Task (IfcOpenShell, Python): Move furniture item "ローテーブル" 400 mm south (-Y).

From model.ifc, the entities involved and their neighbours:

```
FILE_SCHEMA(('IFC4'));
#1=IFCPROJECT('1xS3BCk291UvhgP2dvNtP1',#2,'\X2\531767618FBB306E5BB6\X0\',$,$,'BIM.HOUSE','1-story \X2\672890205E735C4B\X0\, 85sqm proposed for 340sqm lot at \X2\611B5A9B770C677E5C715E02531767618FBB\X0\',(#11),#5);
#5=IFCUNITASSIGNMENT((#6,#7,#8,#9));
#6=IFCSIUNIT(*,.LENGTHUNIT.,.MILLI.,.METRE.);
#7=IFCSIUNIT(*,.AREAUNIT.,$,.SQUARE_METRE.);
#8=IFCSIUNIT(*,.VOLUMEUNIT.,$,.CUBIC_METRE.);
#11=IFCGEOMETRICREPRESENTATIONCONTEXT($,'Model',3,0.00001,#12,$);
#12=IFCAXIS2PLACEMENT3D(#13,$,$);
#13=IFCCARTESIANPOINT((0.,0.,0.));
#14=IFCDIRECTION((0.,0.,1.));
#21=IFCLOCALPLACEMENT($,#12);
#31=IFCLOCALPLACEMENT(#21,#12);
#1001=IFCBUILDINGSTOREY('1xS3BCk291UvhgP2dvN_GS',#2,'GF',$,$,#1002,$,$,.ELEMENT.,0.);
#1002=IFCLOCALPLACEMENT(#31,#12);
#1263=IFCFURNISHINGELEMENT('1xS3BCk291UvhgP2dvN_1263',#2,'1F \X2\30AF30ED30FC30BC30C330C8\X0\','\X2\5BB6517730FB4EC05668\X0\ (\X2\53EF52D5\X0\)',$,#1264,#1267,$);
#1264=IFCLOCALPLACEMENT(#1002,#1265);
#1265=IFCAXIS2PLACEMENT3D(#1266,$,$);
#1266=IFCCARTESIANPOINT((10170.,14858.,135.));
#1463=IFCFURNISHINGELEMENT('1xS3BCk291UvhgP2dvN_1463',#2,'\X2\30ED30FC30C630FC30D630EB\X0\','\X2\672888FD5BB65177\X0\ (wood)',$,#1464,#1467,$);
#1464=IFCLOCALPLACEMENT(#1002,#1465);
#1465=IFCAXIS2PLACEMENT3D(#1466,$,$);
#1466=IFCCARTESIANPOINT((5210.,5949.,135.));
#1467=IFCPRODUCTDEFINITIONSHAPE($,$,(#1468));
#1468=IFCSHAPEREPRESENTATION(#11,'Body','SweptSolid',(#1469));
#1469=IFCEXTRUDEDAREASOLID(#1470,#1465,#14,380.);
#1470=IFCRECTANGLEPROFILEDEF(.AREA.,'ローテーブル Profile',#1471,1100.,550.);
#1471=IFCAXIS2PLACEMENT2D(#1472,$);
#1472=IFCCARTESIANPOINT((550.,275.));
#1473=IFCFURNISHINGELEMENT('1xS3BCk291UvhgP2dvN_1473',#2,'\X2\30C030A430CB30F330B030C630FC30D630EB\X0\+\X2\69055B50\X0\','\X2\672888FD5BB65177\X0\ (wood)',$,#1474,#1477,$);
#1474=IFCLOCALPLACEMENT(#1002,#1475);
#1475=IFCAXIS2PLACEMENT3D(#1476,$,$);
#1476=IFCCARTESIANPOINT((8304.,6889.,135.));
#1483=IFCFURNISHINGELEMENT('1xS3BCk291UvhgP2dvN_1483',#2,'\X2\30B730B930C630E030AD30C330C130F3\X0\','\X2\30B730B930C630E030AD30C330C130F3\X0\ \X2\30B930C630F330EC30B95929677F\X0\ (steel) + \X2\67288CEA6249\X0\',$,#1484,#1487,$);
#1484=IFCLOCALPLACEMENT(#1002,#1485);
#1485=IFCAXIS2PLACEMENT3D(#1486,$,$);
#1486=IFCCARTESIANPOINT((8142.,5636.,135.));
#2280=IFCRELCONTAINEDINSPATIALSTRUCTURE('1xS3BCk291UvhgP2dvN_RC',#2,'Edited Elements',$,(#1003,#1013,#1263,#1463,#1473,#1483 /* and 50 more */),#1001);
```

```python
import ifcopenshell
import ifcopenshell.api.geometry
import ifcopenshell.util.placement
import ifcopenshell.util.unit

model = ifcopenshell.open("model.ifc")
unit_scale = ifcopenshell.util.unit.calculate_unit_scale(model)

item = model.by_guid("1xS3BCk291UvhgP2dvN_1463")
matrix = ifcopenshell.util.placement.get_local_placement(item.ObjectPlacement)
matrix[1, 3] -= 0.4 / unit_scale
ifcopenshell.api.geometry.edit_object_placement(model, product=item, matrix=matrix, is_si=False)

print(ifcopenshell.util.placement.get_local_placement(item.ObjectPlacement).round(3) + 0.0)

model.write("model_v2.ifc")
```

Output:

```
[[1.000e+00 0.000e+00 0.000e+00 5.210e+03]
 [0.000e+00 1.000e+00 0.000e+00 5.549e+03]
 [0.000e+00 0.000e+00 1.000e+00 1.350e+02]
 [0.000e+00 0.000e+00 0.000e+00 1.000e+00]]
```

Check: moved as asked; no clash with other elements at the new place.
